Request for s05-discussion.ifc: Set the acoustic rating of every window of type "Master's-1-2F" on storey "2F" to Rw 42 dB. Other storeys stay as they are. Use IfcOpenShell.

First a look at what the model holds.

```python
import ifcopenshell
import ifcopenshell.util.element

model = ifcopenshell.open("s05-discussion.ifc")
print(model.schema)
storey = next(s for s in model.by_type("IfcBuildingStorey") if s.Name == "2F")
windows = [e for e in ifcopenshell.util.element.get_decomposition(storey) if e.is_a("IfcWindow")]
seen = {}
for e in windows:
    element_type = ifcopenshell.util.element.get_type(e)
    key = (element_type.Name if element_type != e and element_type else None, ifcopenshell.util.element.get_pset(e, "Pset_WindowCommon", "AcousticRating"))
    seen[key] = seen.get(key, 0) + 1
for (name, value), count in sorted(seen.items(), key=str):
    print(count, "x", name, "|", value)
```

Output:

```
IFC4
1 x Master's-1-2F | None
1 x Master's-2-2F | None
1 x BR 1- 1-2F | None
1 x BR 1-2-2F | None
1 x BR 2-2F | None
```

```python
import ifcopenshell
import ifcopenshell.api.pset
import ifcopenshell.util.element

model = ifcopenshell.open("s05-discussion.ifc")

storey = next(s for s in model.by_type("IfcBuildingStorey") if s.Name == "2F")
windows = [e for e in ifcopenshell.util.element.get_decomposition(storey) if e.is_a("IfcWindow")]

count = 0
for e in windows:
    element_type = ifcopenshell.util.element.get_type(e)
    if element_type in (None, e) or element_type.Name != "Master's-1-2F":
        continue
    # add_pset returns the element's existing set when there is one.
    pset = ifcopenshell.api.pset.add_pset(model, product=e, name="Pset_WindowCommon")
    ifcopenshell.api.pset.edit_pset(model, pset=pset, properties={"AcousticRating": "Rw 42 dB"})
    count += 1

print(count, "windows updated")

model.write("s05-discussion_updated.ifc")
```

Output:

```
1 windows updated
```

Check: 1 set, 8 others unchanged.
